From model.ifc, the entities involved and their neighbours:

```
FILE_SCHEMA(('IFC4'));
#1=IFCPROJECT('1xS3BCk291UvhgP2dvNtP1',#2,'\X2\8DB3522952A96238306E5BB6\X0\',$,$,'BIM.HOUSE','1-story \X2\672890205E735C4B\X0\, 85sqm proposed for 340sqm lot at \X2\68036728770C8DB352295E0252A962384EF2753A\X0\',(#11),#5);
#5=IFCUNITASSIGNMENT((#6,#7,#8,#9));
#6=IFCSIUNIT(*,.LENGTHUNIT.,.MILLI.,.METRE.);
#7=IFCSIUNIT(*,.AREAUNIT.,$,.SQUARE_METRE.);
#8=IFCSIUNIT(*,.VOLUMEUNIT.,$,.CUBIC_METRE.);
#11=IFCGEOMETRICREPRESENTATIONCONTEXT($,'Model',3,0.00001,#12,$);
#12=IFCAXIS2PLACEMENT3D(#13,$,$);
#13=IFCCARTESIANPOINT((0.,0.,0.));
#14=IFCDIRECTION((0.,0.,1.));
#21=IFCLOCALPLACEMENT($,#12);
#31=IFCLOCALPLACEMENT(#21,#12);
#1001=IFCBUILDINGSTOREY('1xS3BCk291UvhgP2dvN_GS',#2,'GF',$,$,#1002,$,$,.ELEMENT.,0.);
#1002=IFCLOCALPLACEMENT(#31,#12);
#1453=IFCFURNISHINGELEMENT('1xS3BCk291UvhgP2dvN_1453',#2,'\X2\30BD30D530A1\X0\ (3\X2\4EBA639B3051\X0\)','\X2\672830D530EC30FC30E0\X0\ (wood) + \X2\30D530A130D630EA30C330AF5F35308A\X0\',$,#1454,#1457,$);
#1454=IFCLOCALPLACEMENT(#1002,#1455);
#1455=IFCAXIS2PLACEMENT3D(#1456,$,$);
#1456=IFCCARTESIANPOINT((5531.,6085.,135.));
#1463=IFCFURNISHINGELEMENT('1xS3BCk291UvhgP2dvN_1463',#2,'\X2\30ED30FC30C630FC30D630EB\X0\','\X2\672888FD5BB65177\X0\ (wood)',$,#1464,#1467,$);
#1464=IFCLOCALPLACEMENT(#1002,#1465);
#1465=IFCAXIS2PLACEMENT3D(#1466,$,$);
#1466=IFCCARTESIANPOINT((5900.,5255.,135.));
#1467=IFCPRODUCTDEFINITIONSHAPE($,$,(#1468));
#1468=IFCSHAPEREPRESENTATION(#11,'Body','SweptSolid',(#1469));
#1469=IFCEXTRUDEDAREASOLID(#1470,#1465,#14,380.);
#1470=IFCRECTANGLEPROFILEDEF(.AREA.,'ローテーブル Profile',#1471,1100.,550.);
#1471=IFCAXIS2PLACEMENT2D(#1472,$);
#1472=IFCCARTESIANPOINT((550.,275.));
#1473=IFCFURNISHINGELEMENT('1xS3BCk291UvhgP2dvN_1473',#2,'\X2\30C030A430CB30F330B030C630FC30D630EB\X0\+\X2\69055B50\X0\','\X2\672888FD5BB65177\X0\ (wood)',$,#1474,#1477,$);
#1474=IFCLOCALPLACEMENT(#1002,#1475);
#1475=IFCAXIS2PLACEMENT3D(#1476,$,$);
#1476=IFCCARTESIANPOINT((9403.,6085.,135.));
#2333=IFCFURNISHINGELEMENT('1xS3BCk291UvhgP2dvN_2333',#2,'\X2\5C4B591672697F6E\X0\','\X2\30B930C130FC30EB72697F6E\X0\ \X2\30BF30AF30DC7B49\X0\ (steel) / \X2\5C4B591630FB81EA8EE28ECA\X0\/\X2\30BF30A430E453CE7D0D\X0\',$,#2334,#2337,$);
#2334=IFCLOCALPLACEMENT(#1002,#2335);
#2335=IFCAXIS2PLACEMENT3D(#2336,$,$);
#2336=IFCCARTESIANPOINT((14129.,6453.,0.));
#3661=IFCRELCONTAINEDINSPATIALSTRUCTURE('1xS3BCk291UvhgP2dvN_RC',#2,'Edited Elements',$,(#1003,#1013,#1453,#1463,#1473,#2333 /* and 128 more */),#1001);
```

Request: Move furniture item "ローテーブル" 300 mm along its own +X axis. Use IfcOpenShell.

```python
import ifcopenshell
import ifcopenshell.api.geometry
import ifcopenshell.util.placement
import ifcopenshell.util.unit

model = ifcopenshell.open("model.ifc")
unit_scale = ifcopenshell.util.unit.calculate_unit_scale(model)

item = model.by_guid("1xS3BCk291UvhgP2dvN_1463")
matrix = ifcopenshell.util.placement.get_local_placement(item.ObjectPlacement)
matrix[:3, 3] += matrix[:3, 0] * 0.3 / unit_scale
ifcopenshell.api.geometry.edit_object_placement(model, product=item, matrix=matrix, is_si=False)

print(ifcopenshell.util.placement.get_local_placement(item.ObjectPlacement).round(3) + 0.0)

model.write("model_updated.ifc")
```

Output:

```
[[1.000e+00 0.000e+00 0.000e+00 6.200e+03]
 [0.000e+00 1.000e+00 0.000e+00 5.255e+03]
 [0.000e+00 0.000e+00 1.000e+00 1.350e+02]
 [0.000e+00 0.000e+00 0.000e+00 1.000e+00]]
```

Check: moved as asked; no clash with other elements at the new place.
